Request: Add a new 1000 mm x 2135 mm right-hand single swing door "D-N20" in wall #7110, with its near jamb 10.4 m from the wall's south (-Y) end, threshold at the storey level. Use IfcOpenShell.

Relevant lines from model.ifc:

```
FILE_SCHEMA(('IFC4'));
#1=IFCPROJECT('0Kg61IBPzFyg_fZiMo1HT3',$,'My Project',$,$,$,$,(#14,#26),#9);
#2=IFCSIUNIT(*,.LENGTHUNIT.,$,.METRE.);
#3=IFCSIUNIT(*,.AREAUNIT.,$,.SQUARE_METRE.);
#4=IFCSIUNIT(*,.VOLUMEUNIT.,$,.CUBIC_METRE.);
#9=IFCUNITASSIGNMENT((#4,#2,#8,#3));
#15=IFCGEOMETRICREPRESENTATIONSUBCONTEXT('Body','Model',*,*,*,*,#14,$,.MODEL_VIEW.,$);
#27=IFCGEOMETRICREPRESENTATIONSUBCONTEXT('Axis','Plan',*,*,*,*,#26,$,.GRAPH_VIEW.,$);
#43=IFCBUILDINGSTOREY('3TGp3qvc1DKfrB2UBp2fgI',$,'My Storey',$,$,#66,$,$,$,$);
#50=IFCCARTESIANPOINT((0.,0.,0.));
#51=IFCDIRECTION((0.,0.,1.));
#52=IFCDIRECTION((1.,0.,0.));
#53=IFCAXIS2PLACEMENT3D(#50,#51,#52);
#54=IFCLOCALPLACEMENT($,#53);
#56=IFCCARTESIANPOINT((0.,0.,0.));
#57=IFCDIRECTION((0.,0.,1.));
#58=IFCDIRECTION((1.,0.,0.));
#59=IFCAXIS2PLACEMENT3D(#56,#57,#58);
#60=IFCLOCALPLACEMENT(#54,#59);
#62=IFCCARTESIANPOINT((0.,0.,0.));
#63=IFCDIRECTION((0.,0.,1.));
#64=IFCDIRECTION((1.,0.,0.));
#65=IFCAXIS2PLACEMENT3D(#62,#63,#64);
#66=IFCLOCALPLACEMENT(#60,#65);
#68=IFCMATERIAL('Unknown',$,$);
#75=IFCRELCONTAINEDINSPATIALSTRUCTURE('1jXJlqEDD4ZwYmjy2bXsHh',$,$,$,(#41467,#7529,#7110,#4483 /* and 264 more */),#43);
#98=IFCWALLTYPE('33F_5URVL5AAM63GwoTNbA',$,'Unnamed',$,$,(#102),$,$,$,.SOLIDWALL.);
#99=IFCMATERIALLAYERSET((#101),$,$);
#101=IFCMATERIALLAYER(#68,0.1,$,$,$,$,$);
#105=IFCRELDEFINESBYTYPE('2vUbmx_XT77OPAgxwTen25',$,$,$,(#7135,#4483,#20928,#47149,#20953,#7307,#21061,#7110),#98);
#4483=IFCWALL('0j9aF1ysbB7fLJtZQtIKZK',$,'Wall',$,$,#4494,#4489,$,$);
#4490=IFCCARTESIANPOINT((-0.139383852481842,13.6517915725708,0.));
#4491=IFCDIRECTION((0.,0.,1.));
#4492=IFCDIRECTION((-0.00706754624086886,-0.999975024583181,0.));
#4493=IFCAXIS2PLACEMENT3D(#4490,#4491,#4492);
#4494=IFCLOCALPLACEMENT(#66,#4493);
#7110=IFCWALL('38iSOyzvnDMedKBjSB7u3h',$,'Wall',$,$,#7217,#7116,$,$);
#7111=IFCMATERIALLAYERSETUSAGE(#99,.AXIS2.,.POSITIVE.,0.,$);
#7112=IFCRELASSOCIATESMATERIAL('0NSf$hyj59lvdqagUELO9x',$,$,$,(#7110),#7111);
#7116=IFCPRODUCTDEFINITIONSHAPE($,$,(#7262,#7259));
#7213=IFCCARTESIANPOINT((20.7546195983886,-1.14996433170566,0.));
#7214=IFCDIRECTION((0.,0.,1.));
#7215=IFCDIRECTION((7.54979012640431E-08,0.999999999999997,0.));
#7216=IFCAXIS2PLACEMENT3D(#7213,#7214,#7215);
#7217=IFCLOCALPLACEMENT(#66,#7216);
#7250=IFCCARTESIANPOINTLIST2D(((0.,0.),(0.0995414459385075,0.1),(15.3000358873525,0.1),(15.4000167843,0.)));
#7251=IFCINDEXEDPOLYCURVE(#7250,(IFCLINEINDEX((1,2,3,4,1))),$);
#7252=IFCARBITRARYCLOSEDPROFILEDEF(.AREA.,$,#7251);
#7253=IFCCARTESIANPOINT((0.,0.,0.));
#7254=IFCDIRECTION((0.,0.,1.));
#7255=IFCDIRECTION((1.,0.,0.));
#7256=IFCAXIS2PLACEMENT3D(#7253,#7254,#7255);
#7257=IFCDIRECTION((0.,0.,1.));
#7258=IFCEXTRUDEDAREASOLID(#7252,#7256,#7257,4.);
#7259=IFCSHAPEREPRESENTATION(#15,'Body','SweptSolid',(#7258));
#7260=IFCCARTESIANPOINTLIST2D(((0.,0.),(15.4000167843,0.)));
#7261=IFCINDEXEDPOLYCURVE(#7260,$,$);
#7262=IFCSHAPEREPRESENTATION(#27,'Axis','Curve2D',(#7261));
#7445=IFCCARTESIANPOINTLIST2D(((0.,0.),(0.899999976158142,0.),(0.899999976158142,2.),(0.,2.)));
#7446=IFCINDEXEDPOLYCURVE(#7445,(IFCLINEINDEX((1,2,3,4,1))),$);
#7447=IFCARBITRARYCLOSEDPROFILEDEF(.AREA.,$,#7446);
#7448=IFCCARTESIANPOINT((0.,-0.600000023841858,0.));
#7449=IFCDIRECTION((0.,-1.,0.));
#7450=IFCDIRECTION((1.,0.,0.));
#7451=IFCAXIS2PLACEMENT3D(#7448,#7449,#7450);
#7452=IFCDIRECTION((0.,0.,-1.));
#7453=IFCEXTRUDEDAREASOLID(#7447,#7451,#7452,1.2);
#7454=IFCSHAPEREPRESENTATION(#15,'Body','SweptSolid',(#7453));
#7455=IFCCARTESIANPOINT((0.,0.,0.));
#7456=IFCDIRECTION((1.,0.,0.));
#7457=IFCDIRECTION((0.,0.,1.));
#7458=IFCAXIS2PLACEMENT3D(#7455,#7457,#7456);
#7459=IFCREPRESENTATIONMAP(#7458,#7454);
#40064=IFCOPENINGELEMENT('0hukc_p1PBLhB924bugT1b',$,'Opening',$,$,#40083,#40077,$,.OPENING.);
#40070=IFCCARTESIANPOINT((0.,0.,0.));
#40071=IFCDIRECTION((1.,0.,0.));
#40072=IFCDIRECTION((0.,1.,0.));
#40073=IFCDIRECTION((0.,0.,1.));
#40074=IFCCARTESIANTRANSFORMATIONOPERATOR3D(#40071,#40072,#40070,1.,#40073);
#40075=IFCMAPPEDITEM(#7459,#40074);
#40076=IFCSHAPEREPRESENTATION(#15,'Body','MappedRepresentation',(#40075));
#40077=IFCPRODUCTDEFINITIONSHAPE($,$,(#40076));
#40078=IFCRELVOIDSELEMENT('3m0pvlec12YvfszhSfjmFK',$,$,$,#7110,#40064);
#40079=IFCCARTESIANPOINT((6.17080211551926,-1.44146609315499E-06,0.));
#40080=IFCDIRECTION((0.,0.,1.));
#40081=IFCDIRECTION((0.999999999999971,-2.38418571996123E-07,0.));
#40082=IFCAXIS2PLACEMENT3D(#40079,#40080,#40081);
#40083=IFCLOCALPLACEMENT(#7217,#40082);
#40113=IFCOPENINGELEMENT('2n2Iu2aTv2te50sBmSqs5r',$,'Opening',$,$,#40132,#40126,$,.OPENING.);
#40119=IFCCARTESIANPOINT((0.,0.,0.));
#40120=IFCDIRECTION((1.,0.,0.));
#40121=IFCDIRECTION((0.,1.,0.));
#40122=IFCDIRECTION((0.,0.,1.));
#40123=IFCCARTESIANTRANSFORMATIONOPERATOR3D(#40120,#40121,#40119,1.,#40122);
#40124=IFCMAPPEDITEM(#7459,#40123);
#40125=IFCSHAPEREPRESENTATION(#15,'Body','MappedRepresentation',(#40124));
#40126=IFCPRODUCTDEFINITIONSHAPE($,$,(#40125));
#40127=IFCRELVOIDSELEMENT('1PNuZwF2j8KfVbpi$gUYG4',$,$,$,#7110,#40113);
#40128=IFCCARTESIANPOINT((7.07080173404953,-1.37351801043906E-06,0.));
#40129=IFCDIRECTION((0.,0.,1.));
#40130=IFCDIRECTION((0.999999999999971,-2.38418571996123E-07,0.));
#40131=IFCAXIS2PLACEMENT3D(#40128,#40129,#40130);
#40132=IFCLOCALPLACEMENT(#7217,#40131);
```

```python
import numpy as np
import ifcopenshell
import ifcopenshell.api.feature
import ifcopenshell.api.geometry
import ifcopenshell.api.root
import ifcopenshell.api.spatial
import ifcopenshell.geom
import ifcopenshell.util.element
import ifcopenshell.util.placement
import ifcopenshell.util.representation
import ifcopenshell.util.shape
import ifcopenshell.util.unit

model = ifcopenshell.open("model.ifc")
unit_scale = ifcopenshell.util.unit.calculate_unit_scale(model)
settings = ifcopenshell.geom.settings()


def volume(element):
    """Net volume in cubic metres, openings subtracted."""
    shape = ifcopenshell.geom.create_shape(settings, element)
    return ifcopenshell.util.shape.get_volume(shape.geometry)


wall = model.by_id(7110)
storey = ifcopenshell.util.element.get_container(wall, ifc_class="IfcBuildingStorey")
context = ifcopenshell.util.representation.get_context(model, "Model", "Body", "MODEL_VIEW")
before = volume(wall)

width, height, from_end, sill = 1, 2.135, 10.4, 0.0  # metres

# The wall runs along its own X axis, and the end named is its -X end.
wall_shape = ifcopenshell.geom.create_shape(settings, wall)
x, y, z = ifcopenshell.util.shape.get_vertices(wall_shape.geometry).T
start = x.min() + from_end
face, thickness = float(y.min()), float(y.max() - y.min())
wall_matrix = ifcopenshell.util.placement.get_local_placement(wall.ObjectPlacement)
level = ifcopenshell.util.placement.get_local_placement(storey.ObjectPlacement)[2, 3]


def in_wall(x, y):
    """Placement at x, y metres in the wall's axes, at sill height."""
    matrix = wall_matrix.copy()
    matrix[:, 3] = wall_matrix @ np.array([x / unit_scale, y / unit_scale, 0.0, 1.0])
    matrix[2, 3] = level + sill / unit_scale
    return matrix


# Opening: a box that overshoots both wall faces by 50 mm.
opening = ifcopenshell.api.root.create_entity(model, ifc_class="IfcOpeningElement", predefined_type="OPENING")
box = ifcopenshell.api.geometry.add_wall_representation(
    model, context=context, length=width, height=height, thickness=thickness + 0.1
)
ifcopenshell.api.geometry.assign_representation(model, product=opening, representation=box)
ifcopenshell.api.geometry.edit_object_placement(model, product=opening, matrix=in_wall(start, face - 0.05), is_si=False)
ifcopenshell.api.feature.add_feature(model, feature=opening, element=wall)

door = ifcopenshell.api.root.create_entity(model, ifc_class="IfcDoor", name="D-N20", predefined_type="DOOR")
door.OverallWidth, door.OverallHeight = width / unit_scale, height / unit_scale
door.OperationType = "SINGLE_SWING_RIGHT"
body = ifcopenshell.api.geometry.add_door_representation(
    model,
    context=context,
    overall_width=door.OverallWidth,
    overall_height=door.OverallHeight,
    operation_type="SINGLE_SWING_RIGHT",
    lining_properties={"LiningDepth": thickness / unit_scale, "ThresholdDepth": thickness / unit_scale},
)
ifcopenshell.api.geometry.assign_representation(model, product=door, representation=body)
ifcopenshell.api.spatial.assign_container(model, products=[door], relating_structure=storey)
ifcopenshell.api.feature.add_filling(model, opening=opening, element=door)

# The lining spans the wall, so the door starts at the wall face.
ifcopenshell.api.geometry.edit_object_placement(model, product=door, matrix=in_wall(start, face), is_si=False)

after = volume(wall)

print(f"wall volume {before:.3f} -> {after:.3f} m3")

model.write("model_edited.ifc")
```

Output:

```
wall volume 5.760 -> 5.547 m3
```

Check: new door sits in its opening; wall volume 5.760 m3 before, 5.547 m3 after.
